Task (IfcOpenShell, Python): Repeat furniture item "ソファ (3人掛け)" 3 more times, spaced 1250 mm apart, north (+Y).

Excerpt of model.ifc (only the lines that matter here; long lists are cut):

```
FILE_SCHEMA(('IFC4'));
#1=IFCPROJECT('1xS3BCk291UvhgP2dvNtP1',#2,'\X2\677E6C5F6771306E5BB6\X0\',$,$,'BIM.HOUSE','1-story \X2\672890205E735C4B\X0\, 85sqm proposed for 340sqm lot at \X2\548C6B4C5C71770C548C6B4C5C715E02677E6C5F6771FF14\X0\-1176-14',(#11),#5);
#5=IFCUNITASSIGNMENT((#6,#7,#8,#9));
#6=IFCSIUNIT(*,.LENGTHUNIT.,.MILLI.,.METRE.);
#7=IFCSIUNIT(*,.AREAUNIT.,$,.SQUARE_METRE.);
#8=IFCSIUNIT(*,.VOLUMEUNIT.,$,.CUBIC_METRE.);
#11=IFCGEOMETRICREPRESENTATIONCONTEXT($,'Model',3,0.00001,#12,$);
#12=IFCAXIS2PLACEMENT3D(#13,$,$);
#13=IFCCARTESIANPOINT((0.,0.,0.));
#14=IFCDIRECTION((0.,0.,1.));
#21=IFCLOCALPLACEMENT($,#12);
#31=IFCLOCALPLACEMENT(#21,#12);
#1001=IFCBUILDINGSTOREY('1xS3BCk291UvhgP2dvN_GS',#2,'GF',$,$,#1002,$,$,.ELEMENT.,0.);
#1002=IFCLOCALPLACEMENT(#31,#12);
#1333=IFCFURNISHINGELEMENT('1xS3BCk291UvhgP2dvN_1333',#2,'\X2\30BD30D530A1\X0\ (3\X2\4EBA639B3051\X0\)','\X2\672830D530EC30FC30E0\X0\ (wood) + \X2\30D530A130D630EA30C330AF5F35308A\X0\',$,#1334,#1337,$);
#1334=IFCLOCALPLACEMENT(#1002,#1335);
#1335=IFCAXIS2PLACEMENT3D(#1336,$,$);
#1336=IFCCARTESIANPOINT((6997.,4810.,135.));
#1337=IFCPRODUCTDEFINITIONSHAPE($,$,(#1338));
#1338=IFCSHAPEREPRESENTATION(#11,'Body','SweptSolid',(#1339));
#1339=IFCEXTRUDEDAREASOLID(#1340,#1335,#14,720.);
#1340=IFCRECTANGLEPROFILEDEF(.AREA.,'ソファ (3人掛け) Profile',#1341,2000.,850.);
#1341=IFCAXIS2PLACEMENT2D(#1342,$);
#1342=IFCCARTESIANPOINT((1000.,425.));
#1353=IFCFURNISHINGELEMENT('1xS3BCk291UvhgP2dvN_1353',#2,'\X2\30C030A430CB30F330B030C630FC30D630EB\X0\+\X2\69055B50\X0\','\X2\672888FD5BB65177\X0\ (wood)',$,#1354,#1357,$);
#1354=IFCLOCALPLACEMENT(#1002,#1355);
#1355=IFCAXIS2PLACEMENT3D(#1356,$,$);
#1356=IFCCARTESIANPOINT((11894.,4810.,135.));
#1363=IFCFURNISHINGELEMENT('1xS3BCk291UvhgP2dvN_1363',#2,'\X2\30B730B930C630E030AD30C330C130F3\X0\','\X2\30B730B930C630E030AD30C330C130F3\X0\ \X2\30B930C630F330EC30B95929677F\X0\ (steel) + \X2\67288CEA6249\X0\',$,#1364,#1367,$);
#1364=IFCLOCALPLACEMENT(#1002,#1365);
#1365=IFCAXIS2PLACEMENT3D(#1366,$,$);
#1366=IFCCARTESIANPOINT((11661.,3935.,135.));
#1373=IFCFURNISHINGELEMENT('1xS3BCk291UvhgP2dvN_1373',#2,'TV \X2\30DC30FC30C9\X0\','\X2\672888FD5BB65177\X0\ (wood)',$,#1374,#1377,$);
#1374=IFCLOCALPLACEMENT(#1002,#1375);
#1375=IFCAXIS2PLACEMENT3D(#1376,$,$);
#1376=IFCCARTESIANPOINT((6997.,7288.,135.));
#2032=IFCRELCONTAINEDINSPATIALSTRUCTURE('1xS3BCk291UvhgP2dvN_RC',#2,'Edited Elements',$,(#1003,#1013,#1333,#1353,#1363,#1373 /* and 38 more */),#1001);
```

```python
import numpy as np
import ifcopenshell
import ifcopenshell.api.geometry
import ifcopenshell.api.root
import ifcopenshell.util.element
import ifcopenshell.util.placement

model = ifcopenshell.open("model.ifc")


def reuse_history(source, copy):
    """copy_class also copies each property set's owner history, people and application; keep the originals."""
    for rel in copy.IsDefinedBy:
        if rel.is_a("IfcRelDefinesByProperties") and (history := rel.RelatingPropertyDefinition.OwnerHistory):
            rel.RelatingPropertyDefinition.OwnerHistory = source.OwnerHistory
            ifcopenshell.util.element.remove_deep2(model, history)


source = model.by_guid("1xS3BCk291UvhgP2dvN_1333")
base = ifcopenshell.util.placement.get_local_placement(source.ObjectPlacement)
step = np.array([0.0, 1.0, 0.0]) * 1250.0

for i in range(1, 4):
    copy = ifcopenshell.api.root.copy_class(model, product=source)
    copy.Representation = ifcopenshell.util.element.copy_deep(
        model, source.Representation, exclude=["IfcGeometricRepresentationContext", "IfcRepresentationMap"]
    )
    reuse_history(source, copy)
    matrix = base.copy()
    matrix[:3, 3] += i * step
    print("added at", matrix[:3, 3].round(3) + 0.0)
    ifcopenshell.api.geometry.edit_object_placement(model, product=copy, matrix=matrix, is_si=False)

model.write("model_edited.ifc")
```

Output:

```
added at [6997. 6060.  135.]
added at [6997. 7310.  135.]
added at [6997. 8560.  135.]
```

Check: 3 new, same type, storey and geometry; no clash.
